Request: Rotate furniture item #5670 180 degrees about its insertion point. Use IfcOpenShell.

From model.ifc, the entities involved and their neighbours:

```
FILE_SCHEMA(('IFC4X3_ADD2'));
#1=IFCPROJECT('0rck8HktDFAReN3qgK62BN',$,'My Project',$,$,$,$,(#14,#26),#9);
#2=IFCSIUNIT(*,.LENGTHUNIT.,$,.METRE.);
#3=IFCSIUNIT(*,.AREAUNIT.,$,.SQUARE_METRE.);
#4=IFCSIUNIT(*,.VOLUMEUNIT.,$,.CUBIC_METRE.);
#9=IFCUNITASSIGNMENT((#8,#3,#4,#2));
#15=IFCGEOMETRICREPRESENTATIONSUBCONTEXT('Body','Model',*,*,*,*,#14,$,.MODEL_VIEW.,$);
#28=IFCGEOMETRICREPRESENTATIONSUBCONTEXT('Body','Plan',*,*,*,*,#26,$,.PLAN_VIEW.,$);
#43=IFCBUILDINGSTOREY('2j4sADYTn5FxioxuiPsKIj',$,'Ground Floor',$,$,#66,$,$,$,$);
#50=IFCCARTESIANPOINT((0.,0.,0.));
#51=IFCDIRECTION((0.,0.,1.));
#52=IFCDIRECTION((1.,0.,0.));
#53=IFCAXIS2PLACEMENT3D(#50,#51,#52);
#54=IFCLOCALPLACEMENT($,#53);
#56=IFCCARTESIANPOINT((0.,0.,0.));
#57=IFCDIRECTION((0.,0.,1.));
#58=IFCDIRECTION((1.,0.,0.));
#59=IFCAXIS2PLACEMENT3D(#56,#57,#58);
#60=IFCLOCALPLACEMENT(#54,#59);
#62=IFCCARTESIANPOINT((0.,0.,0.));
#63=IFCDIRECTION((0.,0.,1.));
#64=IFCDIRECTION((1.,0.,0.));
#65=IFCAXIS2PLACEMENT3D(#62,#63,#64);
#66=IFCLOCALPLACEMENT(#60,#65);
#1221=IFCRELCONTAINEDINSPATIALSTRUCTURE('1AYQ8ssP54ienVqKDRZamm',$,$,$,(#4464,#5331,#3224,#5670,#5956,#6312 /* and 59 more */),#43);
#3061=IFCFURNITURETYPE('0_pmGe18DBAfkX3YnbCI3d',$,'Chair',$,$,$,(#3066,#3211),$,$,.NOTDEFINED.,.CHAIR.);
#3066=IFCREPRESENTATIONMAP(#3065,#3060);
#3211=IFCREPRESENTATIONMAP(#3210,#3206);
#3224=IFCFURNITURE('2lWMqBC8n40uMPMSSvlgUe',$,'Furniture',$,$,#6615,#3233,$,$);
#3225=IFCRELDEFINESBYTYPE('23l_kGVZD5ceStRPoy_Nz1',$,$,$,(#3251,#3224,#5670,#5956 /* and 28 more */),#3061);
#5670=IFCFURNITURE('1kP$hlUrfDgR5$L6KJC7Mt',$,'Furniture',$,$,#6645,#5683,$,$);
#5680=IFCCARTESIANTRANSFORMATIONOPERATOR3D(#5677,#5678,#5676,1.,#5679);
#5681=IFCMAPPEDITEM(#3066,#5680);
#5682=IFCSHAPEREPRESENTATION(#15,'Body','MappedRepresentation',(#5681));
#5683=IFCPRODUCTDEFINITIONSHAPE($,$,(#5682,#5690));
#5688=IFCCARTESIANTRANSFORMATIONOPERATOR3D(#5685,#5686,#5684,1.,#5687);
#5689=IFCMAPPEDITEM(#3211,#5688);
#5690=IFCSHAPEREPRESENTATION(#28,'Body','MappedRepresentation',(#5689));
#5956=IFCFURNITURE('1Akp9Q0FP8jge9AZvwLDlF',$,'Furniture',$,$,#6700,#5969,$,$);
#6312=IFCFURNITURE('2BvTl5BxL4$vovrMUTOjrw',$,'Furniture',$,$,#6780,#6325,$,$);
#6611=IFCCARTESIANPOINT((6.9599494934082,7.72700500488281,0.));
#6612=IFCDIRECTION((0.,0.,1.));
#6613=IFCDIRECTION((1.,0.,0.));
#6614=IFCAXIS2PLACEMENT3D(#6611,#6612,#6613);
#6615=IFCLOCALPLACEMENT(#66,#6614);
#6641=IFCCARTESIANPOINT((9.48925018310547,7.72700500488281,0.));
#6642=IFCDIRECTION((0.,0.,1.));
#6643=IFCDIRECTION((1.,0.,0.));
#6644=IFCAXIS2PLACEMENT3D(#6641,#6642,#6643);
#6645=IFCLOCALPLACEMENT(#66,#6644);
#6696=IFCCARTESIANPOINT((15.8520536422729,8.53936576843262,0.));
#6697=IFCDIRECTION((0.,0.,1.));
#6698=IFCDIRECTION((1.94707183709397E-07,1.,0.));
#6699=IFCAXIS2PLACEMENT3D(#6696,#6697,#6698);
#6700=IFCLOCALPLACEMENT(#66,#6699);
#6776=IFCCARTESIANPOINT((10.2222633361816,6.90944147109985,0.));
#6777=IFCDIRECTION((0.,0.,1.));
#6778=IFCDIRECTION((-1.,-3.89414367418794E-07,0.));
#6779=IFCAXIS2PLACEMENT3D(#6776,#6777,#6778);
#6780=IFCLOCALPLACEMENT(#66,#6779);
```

```python
import ifcopenshell
import ifcopenshell.api.geometry
import ifcopenshell.util.placement

model = ifcopenshell.open("model.ifc")

item = model.by_id(5670)
matrix = ifcopenshell.util.placement.get_local_placement(item.ObjectPlacement)
matrix = matrix @ ifcopenshell.util.placement.rotation(180, "Z")
ifcopenshell.api.geometry.edit_object_placement(model, product=item, matrix=matrix, is_si=False)

print(ifcopenshell.util.placement.get_local_placement(item.ObjectPlacement).round(3) + 0.0)

model.write("model_rev.ifc")
```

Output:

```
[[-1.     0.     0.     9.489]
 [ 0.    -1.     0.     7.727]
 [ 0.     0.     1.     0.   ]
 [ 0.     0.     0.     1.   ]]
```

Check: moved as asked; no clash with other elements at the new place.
